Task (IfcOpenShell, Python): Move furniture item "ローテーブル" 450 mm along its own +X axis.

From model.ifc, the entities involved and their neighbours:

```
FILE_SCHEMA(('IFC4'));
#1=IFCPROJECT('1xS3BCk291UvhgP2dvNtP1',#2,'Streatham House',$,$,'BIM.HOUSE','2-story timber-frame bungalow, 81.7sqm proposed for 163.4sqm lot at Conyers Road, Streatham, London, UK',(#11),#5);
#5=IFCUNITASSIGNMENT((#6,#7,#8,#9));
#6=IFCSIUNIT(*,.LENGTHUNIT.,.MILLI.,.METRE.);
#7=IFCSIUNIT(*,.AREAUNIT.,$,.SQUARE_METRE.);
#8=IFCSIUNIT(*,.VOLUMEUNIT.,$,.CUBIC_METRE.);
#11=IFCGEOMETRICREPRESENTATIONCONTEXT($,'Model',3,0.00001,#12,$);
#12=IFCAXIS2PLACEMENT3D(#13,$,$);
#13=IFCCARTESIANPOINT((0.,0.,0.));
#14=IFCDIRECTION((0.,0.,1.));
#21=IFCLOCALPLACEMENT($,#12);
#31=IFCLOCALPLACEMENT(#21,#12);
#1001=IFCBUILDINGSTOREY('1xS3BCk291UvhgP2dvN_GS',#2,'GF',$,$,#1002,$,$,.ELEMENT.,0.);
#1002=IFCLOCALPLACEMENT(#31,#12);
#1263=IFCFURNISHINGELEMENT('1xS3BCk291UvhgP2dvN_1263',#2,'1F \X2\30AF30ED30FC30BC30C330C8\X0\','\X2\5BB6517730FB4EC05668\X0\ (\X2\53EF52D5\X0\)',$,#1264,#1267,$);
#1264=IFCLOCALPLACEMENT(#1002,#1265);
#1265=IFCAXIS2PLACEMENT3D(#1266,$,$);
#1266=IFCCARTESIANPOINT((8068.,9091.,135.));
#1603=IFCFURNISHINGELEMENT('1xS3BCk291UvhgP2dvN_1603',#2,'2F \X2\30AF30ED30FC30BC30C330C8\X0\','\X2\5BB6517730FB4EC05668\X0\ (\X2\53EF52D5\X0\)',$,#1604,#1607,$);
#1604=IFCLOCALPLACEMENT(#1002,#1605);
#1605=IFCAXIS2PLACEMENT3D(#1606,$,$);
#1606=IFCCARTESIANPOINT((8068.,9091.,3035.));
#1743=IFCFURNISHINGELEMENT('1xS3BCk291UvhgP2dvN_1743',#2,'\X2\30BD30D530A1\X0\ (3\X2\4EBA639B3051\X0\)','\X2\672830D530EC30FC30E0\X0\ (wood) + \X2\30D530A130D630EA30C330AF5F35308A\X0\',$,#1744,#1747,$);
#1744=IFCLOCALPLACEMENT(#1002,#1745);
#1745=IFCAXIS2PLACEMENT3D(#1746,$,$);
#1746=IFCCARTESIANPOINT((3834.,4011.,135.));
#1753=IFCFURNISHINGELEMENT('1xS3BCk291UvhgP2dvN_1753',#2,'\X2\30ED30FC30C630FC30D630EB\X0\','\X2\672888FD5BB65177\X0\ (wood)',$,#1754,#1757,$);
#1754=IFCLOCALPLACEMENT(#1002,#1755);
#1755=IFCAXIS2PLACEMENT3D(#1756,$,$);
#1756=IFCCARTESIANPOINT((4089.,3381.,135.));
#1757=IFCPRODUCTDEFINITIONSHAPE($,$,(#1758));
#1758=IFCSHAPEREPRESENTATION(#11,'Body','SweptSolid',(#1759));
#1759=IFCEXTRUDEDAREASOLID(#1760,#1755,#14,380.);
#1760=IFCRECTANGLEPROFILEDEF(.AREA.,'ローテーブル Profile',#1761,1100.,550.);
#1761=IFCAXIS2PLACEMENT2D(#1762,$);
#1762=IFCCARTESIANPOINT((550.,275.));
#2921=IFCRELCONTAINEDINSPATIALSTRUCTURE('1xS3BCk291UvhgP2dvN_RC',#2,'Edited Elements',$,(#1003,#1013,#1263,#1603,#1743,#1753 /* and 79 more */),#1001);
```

```python
import ifcopenshell
import ifcopenshell.api.geometry
import ifcopenshell.util.placement
import ifcopenshell.util.unit

model = ifcopenshell.open("model.ifc")
unit_scale = ifcopenshell.util.unit.calculate_unit_scale(model)

item = model.by_guid("1xS3BCk291UvhgP2dvN_1753")
matrix = ifcopenshell.util.placement.get_local_placement(item.ObjectPlacement)
matrix[:3, 3] += matrix[:3, 0] * 0.45 / unit_scale
ifcopenshell.api.geometry.edit_object_placement(model, product=item, matrix=matrix, is_si=False)

print(ifcopenshell.util.placement.get_local_placement(item.ObjectPlacement).round(3) + 0.0)

model.write("model-out.ifc")
```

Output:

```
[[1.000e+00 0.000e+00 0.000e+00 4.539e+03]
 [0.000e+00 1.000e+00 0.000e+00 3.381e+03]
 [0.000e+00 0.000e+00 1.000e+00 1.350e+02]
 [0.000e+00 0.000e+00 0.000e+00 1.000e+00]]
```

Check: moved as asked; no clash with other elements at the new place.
